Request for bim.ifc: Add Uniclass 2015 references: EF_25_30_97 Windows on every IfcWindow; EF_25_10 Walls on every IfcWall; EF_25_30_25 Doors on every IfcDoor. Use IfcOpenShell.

First a look at what the model holds.

```python
import ifcopenshell

model = ifcopenshell.open("bim.ifc")
print(model.schema)
print("classifications:", [c.Name for c in model.by_type("IfcClassification")])
for ifc_class in ("IfcDoor", "IfcRoof", "IfcStair", "IfcWall", "IfcWindow"):
    print(ifc_class, len(model.by_type(ifc_class)))
```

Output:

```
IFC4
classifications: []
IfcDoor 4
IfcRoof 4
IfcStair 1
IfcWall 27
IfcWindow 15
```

```python
import ifcopenshell
import ifcopenshell.api.classification

model = ifcopenshell.open("bim.ifc")

system = ifcopenshell.api.classification.add_classification(model, classification="Uniclass 2015")

codes = {
    "IfcWindow": ("EF_25_30_97", "Windows"),
    "IfcWall": ("EF_25_10", "Walls"),
    "IfcDoor": ("EF_25_30_25", "Doors"),
}
for ifc_class, (code, name) in codes.items():
    products = model.by_type(ifc_class)
    ifcopenshell.api.classification.add_reference(
        model, products=products, classification=system, identification=code, name=name
    )
    print(code, len(products))

model.write("bim_edited.ifc")
```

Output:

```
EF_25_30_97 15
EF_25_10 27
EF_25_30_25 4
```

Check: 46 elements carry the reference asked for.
